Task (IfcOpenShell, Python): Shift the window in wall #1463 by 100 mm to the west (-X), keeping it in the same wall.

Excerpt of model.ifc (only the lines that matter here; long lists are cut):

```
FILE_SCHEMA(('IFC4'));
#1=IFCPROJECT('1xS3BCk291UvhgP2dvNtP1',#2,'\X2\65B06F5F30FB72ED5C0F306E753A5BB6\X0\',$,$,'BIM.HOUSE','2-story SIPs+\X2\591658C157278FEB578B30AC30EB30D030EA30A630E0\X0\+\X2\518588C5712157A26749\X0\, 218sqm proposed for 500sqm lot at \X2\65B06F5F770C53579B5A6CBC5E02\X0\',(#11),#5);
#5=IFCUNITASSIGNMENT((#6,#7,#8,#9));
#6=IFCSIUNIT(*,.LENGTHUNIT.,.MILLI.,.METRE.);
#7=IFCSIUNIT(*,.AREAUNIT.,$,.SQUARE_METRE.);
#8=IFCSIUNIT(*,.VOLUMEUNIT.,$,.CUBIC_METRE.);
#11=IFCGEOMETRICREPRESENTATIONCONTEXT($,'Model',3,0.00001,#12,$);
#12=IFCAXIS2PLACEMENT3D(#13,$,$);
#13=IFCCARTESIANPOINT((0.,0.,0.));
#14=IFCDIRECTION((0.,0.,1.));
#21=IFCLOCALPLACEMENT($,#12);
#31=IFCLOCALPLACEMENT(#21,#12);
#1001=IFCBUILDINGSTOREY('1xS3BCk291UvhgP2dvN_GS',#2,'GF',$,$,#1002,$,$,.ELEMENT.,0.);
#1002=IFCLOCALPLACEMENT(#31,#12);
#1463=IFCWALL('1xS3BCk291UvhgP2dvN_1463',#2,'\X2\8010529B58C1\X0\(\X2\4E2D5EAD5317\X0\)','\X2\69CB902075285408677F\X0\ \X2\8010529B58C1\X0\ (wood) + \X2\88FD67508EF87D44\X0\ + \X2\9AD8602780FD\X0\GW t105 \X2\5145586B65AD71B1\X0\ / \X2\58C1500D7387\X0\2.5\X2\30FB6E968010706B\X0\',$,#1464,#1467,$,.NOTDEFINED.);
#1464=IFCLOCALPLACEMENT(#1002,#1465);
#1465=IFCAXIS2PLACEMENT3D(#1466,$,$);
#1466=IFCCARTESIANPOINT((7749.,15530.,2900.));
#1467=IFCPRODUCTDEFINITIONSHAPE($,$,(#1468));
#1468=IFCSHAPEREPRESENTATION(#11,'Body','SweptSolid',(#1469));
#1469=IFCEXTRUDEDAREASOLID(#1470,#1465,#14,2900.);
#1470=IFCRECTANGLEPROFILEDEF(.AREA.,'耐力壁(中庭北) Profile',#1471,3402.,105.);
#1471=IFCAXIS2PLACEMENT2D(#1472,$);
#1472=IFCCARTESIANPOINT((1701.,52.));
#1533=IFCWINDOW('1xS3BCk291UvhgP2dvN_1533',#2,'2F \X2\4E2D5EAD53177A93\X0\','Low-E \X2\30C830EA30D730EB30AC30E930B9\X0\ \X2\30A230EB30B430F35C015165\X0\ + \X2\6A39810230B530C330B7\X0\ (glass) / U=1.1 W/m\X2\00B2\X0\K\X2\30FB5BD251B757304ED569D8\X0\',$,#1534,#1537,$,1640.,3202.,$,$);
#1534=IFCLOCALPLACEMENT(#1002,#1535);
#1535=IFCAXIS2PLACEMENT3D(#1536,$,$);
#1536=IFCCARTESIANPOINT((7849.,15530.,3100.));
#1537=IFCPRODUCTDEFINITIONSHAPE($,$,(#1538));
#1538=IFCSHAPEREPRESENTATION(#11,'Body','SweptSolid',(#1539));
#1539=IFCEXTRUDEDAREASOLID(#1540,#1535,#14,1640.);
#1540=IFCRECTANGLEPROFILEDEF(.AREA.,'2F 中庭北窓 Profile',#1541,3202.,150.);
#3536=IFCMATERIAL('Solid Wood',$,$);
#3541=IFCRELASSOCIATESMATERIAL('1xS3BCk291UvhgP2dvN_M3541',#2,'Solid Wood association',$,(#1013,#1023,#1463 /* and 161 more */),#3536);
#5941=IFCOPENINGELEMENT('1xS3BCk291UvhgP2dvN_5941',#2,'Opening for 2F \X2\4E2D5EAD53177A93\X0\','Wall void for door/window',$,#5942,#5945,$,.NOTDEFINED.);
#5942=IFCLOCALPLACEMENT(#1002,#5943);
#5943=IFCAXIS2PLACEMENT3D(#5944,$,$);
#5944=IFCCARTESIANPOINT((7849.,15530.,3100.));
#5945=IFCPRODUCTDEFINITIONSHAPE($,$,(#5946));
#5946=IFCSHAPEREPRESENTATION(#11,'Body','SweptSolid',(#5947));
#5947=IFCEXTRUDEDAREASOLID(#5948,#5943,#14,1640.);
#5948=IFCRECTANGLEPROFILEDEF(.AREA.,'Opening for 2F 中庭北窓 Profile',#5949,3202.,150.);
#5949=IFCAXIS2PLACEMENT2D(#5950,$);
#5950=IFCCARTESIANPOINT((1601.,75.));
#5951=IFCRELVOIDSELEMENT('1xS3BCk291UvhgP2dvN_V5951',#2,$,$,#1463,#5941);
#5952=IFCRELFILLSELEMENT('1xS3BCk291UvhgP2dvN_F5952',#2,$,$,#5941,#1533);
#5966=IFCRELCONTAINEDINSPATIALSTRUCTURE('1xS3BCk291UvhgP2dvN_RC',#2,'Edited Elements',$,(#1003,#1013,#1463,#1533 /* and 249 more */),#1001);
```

```python
import ifcopenshell
import ifcopenshell.api.geometry
import ifcopenshell.util.placement
import ifcopenshell.util.unit

model = ifcopenshell.open("model.ifc")
unit_scale = ifcopenshell.util.unit.calculate_unit_scale(model)

window = model.by_id(1533)
opening = window.FillsVoids[0].RelatingOpeningElement
wall = opening.VoidsElements[0].RelatingBuildingElement

wall_matrix = ifcopenshell.util.placement.get_local_placement(wall.ObjectPlacement)
shift = wall_matrix[:3, 0] * -0.1 / unit_scale
before = ifcopenshell.util.placement.get_local_placement(window.ObjectPlacement)[:3, 3].copy()

# The window is not placed relative to its opening, so move both.
for product in (opening, window):
    matrix = ifcopenshell.util.placement.get_local_placement(product.ObjectPlacement)
    matrix[:3, 3] += shift
    ifcopenshell.api.geometry.edit_object_placement(model, product=product, matrix=matrix, is_si=False)

after = ifcopenshell.util.placement.get_local_placement(window.ObjectPlacement)[:3, 3]
print("window moved by", (after - before).round(3) + 0.0)

model.write("model-out.ifc")
```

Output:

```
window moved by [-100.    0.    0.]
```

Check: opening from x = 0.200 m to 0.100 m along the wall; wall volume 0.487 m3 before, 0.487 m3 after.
